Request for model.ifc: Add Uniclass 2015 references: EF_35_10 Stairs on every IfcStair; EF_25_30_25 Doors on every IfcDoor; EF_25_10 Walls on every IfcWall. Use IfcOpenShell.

First a look at what the model holds.

```python
import ifcopenshell

model = ifcopenshell.open("model.ifc")
print(model.schema)
print("classifications:", [c.Name for c in model.by_type("IfcClassification")])
for ifc_class in ("IfcDoor", "IfcRoof", "IfcStair", "IfcWall", "IfcWindow"):
    print(ifc_class, len(model.by_type(ifc_class)))
```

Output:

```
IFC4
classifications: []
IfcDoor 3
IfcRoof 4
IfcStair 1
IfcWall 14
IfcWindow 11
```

```python
import ifcopenshell
import ifcopenshell.api.classification

model = ifcopenshell.open("model.ifc")

system = ifcopenshell.api.classification.add_classification(model, classification="Uniclass 2015")

codes = {
    "IfcStair": ("EF_35_10", "Stairs"),
    "IfcDoor": ("EF_25_30_25", "Doors"),
    "IfcWall": ("EF_25_10", "Walls"),
}
for ifc_class, (code, name) in codes.items():
    products = model.by_type(ifc_class)
    ifcopenshell.api.classification.add_reference(
        model, products=products, classification=system, identification=code, name=name
    )
    print(code, len(products))

model.write("model_v2.ifc")
```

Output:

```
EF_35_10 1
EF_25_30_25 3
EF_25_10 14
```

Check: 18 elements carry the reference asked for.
